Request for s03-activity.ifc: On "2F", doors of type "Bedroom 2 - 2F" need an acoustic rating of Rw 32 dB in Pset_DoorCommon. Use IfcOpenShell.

First a look at what the model holds.

```python
import ifcopenshell
import ifcopenshell.util.element

model = ifcopenshell.open("s03-activity.ifc")
print(model.schema)
storey = next(s for s in model.by_type("IfcBuildingStorey") if s.Name == "2F")
doors = [e for e in ifcopenshell.util.element.get_decomposition(storey) if e.is_a("IfcDoor")]
seen = {}
for e in doors:
    element_type = ifcopenshell.util.element.get_type(e)
    key = (element_type.Name if element_type != e and element_type else None, ifcopenshell.util.element.get_pset(e, "Pset_DoorCommon", "AcousticRating"))
    seen[key] = seen.get(key, 0) + 1
for (name, value), count in sorted(seen.items(), key=str):
    print(count, "x", name, "|", value)
```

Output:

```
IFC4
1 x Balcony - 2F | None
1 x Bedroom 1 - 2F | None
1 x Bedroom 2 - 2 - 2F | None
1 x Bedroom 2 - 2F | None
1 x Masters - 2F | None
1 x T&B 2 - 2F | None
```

```python
import ifcopenshell
import ifcopenshell.api.pset
import ifcopenshell.util.element

model = ifcopenshell.open("s03-activity.ifc")

storey = next(s for s in model.by_type("IfcBuildingStorey") if s.Name == "2F")
doors = [e for e in ifcopenshell.util.element.get_decomposition(storey) if e.is_a("IfcDoor")]

count = 0
for e in doors:
    element_type = ifcopenshell.util.element.get_type(e)
    if element_type in (None, e) or element_type.Name != "Bedroom 2 - 2F":
        continue
    # add_pset returns the element's existing set when there is one.
    pset = ifcopenshell.api.pset.add_pset(model, product=e, name="Pset_DoorCommon")
    ifcopenshell.api.pset.edit_pset(model, pset=pset, properties={"AcousticRating": "Rw 32 dB"})
    count += 1

print(count, "doors updated")

model.write("s03-activity-out.ifc")
```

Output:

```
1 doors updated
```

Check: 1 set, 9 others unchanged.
